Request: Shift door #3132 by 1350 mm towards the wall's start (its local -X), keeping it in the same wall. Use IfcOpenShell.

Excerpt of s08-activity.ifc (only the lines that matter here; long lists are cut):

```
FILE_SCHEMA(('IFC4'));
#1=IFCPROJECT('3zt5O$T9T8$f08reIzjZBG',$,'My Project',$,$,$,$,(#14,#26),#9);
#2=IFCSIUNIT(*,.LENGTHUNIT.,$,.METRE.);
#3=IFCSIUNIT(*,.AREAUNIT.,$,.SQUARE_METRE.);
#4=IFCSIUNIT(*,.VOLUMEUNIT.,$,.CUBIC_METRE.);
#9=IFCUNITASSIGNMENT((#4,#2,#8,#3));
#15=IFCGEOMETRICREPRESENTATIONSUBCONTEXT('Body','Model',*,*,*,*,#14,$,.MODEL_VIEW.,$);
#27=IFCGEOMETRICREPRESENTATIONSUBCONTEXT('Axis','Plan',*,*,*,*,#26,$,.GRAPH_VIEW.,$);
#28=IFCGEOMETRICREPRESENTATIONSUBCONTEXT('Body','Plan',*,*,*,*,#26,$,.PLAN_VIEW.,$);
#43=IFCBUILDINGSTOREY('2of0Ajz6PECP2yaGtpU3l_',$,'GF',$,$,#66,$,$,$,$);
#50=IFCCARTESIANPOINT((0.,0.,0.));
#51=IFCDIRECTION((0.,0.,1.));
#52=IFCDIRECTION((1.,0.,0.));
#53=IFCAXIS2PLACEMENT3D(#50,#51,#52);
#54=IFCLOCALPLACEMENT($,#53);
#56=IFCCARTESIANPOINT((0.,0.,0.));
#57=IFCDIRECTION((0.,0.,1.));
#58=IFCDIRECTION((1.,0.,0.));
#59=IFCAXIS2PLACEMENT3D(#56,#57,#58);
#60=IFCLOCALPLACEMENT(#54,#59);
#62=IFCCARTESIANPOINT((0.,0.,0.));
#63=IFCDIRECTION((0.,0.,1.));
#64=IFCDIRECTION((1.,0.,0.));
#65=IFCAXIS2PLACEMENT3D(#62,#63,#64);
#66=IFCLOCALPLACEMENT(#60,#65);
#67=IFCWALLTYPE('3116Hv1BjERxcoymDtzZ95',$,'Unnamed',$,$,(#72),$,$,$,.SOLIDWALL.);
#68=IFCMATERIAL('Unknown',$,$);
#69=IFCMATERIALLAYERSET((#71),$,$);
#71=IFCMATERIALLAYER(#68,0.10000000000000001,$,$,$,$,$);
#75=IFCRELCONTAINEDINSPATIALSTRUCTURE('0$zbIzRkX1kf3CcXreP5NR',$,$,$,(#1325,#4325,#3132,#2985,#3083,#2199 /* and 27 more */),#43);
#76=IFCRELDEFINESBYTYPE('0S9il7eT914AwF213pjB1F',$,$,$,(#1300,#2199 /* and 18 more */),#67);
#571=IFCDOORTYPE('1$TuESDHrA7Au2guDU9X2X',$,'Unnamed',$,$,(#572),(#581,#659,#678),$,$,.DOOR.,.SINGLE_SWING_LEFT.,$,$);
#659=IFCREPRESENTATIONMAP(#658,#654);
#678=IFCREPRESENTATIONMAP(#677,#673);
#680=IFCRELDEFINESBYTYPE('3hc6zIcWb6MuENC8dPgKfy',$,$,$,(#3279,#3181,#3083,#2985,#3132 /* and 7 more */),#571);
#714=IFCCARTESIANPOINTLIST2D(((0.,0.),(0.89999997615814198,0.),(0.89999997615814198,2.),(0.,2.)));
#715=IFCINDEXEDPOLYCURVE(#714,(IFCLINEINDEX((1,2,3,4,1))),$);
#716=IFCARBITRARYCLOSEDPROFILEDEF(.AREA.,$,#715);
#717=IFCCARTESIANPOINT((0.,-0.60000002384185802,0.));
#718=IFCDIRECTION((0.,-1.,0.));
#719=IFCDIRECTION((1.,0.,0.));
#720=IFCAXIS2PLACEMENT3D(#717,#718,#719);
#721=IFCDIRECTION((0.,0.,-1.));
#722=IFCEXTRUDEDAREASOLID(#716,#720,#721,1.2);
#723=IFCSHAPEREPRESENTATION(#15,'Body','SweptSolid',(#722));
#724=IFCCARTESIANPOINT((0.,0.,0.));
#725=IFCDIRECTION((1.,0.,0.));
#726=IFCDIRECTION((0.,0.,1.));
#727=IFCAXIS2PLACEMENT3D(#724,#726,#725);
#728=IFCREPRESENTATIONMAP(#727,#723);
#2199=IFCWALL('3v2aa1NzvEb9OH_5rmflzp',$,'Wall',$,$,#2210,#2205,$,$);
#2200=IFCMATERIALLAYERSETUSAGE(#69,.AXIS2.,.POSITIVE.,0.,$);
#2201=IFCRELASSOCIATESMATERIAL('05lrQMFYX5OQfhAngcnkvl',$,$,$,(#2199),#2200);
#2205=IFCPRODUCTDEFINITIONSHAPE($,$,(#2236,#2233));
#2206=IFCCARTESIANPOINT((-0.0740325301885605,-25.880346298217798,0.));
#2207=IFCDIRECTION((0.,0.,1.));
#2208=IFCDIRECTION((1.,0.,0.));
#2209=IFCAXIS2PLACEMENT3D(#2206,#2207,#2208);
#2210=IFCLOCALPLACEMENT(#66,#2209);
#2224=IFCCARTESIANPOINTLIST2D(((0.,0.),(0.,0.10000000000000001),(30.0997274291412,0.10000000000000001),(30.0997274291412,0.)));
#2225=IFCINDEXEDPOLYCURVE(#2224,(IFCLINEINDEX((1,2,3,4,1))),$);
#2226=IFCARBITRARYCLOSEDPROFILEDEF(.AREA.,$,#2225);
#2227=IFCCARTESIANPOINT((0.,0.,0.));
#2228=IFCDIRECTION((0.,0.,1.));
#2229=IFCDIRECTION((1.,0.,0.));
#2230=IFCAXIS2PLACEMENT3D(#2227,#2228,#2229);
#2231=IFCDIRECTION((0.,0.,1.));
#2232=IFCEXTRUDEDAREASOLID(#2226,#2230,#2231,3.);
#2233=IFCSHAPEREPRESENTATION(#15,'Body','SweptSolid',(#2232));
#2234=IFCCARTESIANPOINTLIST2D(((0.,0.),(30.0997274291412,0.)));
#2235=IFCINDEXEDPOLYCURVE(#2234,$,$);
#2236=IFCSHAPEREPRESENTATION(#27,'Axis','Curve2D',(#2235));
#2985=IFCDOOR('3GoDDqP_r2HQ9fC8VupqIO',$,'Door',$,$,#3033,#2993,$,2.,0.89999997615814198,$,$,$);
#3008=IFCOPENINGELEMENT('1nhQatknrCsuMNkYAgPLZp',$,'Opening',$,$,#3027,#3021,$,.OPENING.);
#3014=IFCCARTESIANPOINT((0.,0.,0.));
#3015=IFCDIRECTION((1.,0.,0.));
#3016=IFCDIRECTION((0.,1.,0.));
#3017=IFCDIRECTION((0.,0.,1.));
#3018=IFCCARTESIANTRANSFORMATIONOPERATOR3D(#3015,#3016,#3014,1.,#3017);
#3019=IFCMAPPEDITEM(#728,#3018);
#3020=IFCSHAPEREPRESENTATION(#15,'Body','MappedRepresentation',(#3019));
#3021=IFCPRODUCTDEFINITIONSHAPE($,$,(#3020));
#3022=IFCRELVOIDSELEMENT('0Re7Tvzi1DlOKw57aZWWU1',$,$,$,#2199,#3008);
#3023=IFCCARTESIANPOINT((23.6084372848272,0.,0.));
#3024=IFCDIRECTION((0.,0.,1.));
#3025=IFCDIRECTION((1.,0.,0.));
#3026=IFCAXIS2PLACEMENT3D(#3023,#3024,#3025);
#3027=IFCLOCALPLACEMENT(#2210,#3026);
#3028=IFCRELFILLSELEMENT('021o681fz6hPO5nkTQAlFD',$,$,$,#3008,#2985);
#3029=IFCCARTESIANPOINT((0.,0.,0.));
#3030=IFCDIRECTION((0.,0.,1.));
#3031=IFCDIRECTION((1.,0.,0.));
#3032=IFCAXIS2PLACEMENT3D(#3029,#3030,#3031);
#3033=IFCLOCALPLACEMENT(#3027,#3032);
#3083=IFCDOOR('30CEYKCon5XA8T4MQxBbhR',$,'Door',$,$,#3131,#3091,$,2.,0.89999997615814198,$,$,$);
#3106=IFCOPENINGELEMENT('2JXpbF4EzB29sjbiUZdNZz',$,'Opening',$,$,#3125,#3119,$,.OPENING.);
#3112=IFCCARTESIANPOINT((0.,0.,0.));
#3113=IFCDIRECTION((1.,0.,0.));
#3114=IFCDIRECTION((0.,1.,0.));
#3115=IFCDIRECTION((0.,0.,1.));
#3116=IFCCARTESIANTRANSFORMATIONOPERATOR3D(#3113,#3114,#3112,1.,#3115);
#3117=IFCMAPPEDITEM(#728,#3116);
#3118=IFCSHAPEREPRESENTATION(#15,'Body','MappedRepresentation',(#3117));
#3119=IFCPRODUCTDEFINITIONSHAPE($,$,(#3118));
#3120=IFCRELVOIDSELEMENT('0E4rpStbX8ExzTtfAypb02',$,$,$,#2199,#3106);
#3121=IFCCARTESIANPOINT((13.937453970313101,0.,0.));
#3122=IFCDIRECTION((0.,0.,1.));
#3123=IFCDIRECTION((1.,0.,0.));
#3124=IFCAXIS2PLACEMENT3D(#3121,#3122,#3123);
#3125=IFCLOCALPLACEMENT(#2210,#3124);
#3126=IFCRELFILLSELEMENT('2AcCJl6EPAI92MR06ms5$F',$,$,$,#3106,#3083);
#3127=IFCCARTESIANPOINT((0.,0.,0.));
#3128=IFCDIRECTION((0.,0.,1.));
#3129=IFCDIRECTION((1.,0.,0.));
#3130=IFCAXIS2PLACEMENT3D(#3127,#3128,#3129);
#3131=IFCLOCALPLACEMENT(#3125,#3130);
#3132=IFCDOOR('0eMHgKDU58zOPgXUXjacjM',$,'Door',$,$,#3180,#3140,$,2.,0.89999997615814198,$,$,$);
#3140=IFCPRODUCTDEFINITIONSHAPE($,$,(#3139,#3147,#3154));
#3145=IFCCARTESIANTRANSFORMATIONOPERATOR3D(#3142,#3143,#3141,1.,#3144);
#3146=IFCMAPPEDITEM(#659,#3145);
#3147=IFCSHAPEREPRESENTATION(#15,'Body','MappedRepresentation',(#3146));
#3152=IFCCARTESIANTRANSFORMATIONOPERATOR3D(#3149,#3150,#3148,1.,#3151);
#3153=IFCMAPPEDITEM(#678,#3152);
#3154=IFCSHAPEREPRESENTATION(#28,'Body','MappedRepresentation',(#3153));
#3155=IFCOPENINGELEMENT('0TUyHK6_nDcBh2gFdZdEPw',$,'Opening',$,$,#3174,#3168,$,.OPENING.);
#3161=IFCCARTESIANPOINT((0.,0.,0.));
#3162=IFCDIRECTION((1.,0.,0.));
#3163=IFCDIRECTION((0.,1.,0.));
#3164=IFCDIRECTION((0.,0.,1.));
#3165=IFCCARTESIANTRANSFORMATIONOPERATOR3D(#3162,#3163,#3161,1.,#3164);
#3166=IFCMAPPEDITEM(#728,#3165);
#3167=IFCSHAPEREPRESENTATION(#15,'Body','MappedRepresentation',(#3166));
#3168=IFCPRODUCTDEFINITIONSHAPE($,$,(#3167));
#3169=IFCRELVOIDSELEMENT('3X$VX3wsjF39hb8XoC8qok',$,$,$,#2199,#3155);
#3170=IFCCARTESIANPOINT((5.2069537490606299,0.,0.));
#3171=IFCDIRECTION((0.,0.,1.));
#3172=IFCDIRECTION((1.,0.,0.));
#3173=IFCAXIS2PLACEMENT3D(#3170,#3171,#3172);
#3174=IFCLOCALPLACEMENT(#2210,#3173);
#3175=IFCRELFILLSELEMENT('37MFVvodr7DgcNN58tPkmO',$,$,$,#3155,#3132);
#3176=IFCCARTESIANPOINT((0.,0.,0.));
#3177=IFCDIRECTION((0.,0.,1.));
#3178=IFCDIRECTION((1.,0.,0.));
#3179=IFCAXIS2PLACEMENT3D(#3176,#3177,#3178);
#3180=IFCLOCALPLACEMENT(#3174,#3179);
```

```python
import ifcopenshell
import ifcopenshell.api.geometry
import ifcopenshell.util.placement
import ifcopenshell.util.unit

model = ifcopenshell.open("s08-activity.ifc")
unit_scale = ifcopenshell.util.unit.calculate_unit_scale(model)

door = model.by_guid("0eMHgKDU58zOPgXUXjacjM")
opening = door.FillsVoids[0].RelatingOpeningElement
wall = opening.VoidsElements[0].RelatingBuildingElement

wall_matrix = ifcopenshell.util.placement.get_local_placement(wall.ObjectPlacement)
shift = wall_matrix[:3, 0] * -1.35 / unit_scale
before = ifcopenshell.util.placement.get_local_placement(door.ObjectPlacement)[:3, 3].copy()

# The door is placed relative to its opening, so it follows when the opening moves.
matrix = ifcopenshell.util.placement.get_local_placement(opening.ObjectPlacement)
matrix[:3, 3] += shift
ifcopenshell.api.geometry.edit_object_placement(
    model, product=opening, matrix=matrix, is_si=False, should_transform_children=True
)

after = ifcopenshell.util.placement.get_local_placement(door.ObjectPlacement)[:3, 3]
print("door moved by", (after - before).round(3) + 0.0)

model.write("s08-activity_updated.ifc")
```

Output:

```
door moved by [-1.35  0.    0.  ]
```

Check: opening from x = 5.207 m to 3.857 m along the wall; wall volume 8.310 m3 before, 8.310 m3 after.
